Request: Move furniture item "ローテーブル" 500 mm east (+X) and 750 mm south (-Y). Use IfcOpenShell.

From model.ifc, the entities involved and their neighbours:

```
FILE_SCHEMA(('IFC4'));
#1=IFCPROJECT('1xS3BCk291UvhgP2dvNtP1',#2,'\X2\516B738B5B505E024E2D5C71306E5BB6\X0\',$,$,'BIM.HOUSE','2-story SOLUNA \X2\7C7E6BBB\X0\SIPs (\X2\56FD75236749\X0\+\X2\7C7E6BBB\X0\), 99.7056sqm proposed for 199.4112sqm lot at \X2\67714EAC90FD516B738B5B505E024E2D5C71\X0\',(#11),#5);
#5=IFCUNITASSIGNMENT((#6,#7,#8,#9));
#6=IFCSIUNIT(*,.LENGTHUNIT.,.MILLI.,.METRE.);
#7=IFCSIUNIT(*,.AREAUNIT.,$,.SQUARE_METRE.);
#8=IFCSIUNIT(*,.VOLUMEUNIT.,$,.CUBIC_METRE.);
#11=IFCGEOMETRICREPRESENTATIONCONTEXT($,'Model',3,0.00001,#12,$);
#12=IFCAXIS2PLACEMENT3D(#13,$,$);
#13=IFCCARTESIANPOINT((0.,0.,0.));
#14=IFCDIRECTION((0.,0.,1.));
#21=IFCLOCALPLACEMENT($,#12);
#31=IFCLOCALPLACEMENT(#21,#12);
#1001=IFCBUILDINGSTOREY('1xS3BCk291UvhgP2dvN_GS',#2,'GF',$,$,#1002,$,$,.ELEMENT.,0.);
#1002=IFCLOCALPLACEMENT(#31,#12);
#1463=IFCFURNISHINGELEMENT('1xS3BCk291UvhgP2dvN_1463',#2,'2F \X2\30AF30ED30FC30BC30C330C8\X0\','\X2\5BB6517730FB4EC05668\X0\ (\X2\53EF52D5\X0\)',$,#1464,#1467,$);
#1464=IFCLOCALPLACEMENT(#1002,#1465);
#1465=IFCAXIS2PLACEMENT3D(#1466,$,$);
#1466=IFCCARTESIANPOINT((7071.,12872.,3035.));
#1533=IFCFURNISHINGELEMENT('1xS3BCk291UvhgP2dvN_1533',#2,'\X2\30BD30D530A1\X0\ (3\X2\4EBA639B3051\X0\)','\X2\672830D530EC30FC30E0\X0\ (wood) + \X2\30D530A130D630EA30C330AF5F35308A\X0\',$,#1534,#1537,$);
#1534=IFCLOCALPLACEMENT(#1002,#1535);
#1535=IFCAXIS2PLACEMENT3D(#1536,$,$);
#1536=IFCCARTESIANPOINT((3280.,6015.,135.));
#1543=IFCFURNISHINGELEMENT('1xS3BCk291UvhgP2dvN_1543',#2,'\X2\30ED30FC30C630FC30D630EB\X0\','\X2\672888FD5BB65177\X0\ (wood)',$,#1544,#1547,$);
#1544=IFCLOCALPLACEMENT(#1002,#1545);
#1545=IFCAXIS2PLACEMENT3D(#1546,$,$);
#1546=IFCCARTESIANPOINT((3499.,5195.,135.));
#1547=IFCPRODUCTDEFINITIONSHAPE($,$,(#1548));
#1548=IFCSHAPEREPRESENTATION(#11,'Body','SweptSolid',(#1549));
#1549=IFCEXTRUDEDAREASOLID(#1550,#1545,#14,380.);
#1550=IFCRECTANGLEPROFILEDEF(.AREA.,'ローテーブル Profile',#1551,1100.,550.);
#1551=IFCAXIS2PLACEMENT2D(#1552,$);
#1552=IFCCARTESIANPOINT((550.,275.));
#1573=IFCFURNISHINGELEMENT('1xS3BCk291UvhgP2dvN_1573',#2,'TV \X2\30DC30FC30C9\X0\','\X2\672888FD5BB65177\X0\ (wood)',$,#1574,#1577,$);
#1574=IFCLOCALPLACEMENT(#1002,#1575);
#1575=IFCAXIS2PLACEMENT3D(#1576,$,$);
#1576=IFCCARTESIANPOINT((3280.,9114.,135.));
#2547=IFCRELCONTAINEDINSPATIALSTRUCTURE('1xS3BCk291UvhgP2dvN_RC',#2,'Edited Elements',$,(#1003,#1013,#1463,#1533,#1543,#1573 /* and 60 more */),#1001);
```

```python
import ifcopenshell
import ifcopenshell.api.geometry
import ifcopenshell.util.placement
import ifcopenshell.util.unit

model = ifcopenshell.open("model.ifc")
unit_scale = ifcopenshell.util.unit.calculate_unit_scale(model)

item = model.by_guid("1xS3BCk291UvhgP2dvN_1543")
matrix = ifcopenshell.util.placement.get_local_placement(item.ObjectPlacement)
matrix[0, 3] += 0.5 / unit_scale
matrix[1, 3] -= 0.75 / unit_scale
ifcopenshell.api.geometry.edit_object_placement(model, product=item, matrix=matrix, is_si=False)

print(ifcopenshell.util.placement.get_local_placement(item.ObjectPlacement).round(3) + 0.0)

model.write("model_rev.ifc")
```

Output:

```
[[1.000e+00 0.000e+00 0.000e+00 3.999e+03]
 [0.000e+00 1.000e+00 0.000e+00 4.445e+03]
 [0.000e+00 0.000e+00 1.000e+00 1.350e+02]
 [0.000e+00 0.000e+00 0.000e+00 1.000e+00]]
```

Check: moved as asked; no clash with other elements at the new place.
